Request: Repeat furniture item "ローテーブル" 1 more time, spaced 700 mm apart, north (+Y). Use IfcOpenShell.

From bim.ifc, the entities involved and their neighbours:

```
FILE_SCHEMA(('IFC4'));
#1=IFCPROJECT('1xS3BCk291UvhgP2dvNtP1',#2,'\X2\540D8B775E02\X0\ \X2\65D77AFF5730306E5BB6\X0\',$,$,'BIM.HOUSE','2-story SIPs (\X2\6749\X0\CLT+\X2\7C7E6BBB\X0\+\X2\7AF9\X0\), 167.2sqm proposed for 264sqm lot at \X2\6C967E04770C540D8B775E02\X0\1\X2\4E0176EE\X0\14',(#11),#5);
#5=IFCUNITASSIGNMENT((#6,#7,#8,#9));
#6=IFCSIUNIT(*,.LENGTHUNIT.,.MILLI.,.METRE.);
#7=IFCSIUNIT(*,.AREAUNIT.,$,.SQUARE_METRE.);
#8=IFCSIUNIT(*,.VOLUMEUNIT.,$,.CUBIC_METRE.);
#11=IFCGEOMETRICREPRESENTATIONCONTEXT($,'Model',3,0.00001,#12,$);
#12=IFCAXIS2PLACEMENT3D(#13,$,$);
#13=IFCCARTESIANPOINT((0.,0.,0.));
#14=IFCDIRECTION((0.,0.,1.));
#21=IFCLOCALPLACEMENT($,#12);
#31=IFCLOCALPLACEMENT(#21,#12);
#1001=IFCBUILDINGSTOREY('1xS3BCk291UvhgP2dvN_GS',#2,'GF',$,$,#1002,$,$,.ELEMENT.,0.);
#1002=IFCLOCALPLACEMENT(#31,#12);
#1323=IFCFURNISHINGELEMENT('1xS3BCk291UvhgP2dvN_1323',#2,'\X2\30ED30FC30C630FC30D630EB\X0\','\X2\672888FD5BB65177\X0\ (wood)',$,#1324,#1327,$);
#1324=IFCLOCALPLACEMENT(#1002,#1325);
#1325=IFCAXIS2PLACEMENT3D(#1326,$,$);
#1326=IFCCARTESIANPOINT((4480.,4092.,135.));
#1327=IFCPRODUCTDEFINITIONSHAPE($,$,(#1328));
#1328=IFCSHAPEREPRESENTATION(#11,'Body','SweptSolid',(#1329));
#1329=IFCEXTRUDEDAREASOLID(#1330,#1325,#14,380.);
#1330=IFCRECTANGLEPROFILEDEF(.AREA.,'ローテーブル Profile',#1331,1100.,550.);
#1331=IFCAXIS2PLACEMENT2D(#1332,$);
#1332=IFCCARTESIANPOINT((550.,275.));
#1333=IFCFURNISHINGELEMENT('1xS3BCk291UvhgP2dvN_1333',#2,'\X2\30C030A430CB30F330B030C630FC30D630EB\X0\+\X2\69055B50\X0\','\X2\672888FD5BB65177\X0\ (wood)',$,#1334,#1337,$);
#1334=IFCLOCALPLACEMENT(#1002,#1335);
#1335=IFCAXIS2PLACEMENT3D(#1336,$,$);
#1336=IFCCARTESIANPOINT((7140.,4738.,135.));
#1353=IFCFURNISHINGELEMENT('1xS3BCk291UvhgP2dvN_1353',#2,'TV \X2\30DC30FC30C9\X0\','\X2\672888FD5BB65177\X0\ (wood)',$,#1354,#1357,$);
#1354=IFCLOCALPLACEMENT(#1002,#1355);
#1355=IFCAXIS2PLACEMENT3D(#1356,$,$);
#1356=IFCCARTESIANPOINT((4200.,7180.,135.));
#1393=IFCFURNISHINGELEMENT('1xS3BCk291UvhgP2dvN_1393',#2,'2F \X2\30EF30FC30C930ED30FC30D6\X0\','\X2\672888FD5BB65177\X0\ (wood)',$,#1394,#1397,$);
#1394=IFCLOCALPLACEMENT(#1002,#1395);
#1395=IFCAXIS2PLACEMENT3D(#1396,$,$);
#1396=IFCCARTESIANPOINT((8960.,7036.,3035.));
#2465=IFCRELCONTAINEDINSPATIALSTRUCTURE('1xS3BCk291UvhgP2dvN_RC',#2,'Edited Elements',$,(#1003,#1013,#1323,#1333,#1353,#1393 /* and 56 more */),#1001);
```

```python
import numpy as np
import ifcopenshell
import ifcopenshell.api.geometry
import ifcopenshell.api.root
import ifcopenshell.util.element
import ifcopenshell.util.placement

model = ifcopenshell.open("bim.ifc")


def reuse_history(source, copy):
    """copy_class also copies each property set's owner history, people and application; keep the originals."""
    for rel in copy.IsDefinedBy:
        if rel.is_a("IfcRelDefinesByProperties") and (history := rel.RelatingPropertyDefinition.OwnerHistory):
            rel.RelatingPropertyDefinition.OwnerHistory = source.OwnerHistory
            ifcopenshell.util.element.remove_deep2(model, history)


source = model.by_guid("1xS3BCk291UvhgP2dvN_1323")
base = ifcopenshell.util.placement.get_local_placement(source.ObjectPlacement)
step = np.array([0.0, 1.0, 0.0]) * 700.0

for i in range(1, 2):
    copy = ifcopenshell.api.root.copy_class(model, product=source)
    copy.Representation = ifcopenshell.util.element.copy_deep(
        model, source.Representation, exclude=["IfcGeometricRepresentationContext", "IfcRepresentationMap"]
    )
    reuse_history(source, copy)
    matrix = base.copy()
    matrix[:3, 3] += i * step
    print("added at", matrix[:3, 3].round(3) + 0.0)
    ifcopenshell.api.geometry.edit_object_placement(model, product=copy, matrix=matrix, is_si=False)

model.write("bim_updated.ifc")
```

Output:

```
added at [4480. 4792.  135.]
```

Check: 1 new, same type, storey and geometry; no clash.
